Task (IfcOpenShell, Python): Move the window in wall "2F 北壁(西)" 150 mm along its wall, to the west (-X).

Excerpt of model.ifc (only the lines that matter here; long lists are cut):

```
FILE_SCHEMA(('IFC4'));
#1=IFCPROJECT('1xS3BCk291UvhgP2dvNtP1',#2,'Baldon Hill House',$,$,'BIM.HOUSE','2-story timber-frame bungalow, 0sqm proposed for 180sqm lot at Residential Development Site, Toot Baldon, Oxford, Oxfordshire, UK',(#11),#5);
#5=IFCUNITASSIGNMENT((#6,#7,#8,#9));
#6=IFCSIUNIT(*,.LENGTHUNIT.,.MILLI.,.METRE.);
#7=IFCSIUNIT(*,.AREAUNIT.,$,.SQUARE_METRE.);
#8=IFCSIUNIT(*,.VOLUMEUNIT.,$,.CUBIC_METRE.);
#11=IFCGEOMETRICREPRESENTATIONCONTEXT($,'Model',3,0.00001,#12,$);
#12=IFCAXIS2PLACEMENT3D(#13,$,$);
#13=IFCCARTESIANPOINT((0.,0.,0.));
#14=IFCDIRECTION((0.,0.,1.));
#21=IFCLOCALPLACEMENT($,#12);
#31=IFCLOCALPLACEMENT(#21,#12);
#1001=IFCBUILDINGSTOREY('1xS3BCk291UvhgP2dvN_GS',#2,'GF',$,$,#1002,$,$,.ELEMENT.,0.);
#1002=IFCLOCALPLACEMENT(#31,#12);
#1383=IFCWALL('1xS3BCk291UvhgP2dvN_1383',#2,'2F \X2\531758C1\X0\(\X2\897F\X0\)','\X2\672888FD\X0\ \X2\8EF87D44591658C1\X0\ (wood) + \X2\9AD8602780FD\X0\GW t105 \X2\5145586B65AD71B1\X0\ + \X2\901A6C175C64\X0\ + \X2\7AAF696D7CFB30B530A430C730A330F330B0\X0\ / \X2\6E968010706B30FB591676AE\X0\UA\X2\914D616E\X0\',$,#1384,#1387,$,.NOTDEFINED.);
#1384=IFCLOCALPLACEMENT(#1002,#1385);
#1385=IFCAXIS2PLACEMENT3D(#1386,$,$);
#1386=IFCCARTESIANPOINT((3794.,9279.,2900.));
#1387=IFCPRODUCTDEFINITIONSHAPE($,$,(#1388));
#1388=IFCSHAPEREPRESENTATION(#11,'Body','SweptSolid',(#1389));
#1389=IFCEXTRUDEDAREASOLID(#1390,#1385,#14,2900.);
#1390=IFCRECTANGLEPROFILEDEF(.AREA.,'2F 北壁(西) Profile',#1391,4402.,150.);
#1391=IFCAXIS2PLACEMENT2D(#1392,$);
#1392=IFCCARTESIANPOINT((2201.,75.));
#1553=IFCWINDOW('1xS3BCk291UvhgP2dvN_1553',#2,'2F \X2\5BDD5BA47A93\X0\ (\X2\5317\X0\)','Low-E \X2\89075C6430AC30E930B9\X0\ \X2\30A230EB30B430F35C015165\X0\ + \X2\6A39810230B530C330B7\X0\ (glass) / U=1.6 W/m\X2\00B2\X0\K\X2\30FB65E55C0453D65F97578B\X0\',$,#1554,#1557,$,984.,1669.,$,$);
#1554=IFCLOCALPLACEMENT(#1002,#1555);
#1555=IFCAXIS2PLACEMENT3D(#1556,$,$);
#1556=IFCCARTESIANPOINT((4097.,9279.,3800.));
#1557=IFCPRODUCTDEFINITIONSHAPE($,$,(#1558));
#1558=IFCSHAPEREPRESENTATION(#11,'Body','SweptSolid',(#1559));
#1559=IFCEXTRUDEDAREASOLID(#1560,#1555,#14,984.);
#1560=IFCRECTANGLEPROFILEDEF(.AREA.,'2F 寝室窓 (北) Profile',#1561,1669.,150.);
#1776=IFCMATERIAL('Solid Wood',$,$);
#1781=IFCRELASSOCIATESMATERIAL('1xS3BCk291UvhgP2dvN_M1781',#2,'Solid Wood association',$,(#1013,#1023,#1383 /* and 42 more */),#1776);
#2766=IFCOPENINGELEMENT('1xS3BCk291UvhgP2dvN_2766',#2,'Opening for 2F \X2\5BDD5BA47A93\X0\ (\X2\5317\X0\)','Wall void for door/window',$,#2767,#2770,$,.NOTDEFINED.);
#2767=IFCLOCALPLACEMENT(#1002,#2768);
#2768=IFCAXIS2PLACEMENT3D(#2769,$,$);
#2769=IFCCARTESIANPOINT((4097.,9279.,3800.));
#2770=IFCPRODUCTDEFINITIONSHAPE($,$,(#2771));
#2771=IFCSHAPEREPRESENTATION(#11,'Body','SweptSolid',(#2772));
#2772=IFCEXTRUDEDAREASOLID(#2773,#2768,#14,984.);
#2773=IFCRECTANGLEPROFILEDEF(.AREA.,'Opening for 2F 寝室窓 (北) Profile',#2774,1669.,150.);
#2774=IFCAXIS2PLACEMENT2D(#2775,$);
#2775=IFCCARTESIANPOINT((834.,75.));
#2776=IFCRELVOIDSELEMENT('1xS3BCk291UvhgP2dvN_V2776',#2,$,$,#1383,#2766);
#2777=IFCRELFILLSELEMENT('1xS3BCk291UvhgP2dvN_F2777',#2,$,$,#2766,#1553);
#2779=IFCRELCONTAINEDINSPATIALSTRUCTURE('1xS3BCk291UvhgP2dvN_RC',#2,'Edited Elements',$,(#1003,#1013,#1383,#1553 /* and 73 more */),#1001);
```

```python
import ifcopenshell
import ifcopenshell.api.geometry
import ifcopenshell.util.placement
import ifcopenshell.util.unit

model = ifcopenshell.open("model.ifc")
unit_scale = ifcopenshell.util.unit.calculate_unit_scale(model)

window = model.by_id(1553)
opening = window.FillsVoids[0].RelatingOpeningElement
wall = opening.VoidsElements[0].RelatingBuildingElement

wall_matrix = ifcopenshell.util.placement.get_local_placement(wall.ObjectPlacement)
shift = wall_matrix[:3, 0] * -0.15 / unit_scale
before = ifcopenshell.util.placement.get_local_placement(window.ObjectPlacement)[:3, 3].copy()

# The window is not placed relative to its opening, so move both.
for product in (opening, window):
    matrix = ifcopenshell.util.placement.get_local_placement(product.ObjectPlacement)
    matrix[:3, 3] += shift
    ifcopenshell.api.geometry.edit_object_placement(model, product=product, matrix=matrix, is_si=False)

after = ifcopenshell.util.placement.get_local_placement(window.ObjectPlacement)[:3, 3]
print("window moved by", (after - before).round(3) + 0.0)

model.write("model_rev.ifc")
```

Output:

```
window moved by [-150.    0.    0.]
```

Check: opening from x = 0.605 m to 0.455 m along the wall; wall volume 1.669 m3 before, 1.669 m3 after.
